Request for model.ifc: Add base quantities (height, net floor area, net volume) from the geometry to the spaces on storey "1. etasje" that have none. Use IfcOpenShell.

First a look at what the model holds.

```python
import ifcopenshell
import ifcopenshell.util.element
import ifcopenshell.util.unit

model = ifcopenshell.open("model.ifc")
print(model.schema)
for unit_type in ("LENGTHUNIT", "AREAUNIT", "VOLUMEUNIT"):
    print(unit_type, ifcopenshell.util.unit.calculate_unit_scale(model, unit_type))
storey = next(s for s in model.by_type("IfcBuildingStorey") if s.Name == "1. etasje")
spaces = [e for e in ifcopenshell.util.element.get_decomposition(storey) if e.is_a("IfcSpace")]
for e in sorted(spaces, key=lambda e: e.id()):
    print(e.id(), e.is_a(), e.Name, list(ifcopenshell.util.element.get_psets(e, qtos_only=True)), sep=" | ")
```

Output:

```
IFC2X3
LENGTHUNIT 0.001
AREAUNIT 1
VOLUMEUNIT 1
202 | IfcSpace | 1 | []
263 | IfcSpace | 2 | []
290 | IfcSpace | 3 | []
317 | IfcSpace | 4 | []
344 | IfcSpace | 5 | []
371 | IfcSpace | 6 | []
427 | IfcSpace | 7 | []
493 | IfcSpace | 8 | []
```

```python
import ifcopenshell
import ifcopenshell.api.pset
import ifcopenshell.geom
import ifcopenshell.util.element
import ifcopenshell.util.shape
import ifcopenshell.util.unit

model = ifcopenshell.open("model.ifc")
unit_scale = ifcopenshell.util.unit.calculate_unit_scale(model)
area_scale = ifcopenshell.util.unit.calculate_unit_scale(model, "AREAUNIT")
volume_scale = ifcopenshell.util.unit.calculate_unit_scale(model, "VOLUMEUNIT")
settings = ifcopenshell.geom.settings()

storey = next(s for s in model.by_type("IfcBuildingStorey") if s.Name == "1. etasje")
spaces = [e for e in ifcopenshell.util.element.get_decomposition(storey) if e.is_a("IfcSpace")]

for e in sorted(spaces, key=lambda e: e.id()):
    if ifcopenshell.util.element.get_psets(e, qtos_only=True, should_inherit=False):
        continue
    # Geometry comes back in metres, in the element's own axes.
    shape = ifcopenshell.geom.create_shape(settings, e)
    values = {
        "Height": ifcopenshell.util.shape.get_z(shape.geometry) / unit_scale,
        "NetFloorArea": ifcopenshell.util.shape.get_footprint_area(shape.geometry) / area_scale,
        "NetVolume": ifcopenshell.util.shape.get_volume(shape.geometry) / volume_scale,
    }
    qto = ifcopenshell.api.pset.add_qto(model, product=e, name="BaseQuantities")
    ifcopenshell.api.pset.edit_qto(model, qto=qto, properties=values)
    print(e.id(), {k: round(v, 3) for k, v in values.items()})

model.write("model_edited.ifc")
```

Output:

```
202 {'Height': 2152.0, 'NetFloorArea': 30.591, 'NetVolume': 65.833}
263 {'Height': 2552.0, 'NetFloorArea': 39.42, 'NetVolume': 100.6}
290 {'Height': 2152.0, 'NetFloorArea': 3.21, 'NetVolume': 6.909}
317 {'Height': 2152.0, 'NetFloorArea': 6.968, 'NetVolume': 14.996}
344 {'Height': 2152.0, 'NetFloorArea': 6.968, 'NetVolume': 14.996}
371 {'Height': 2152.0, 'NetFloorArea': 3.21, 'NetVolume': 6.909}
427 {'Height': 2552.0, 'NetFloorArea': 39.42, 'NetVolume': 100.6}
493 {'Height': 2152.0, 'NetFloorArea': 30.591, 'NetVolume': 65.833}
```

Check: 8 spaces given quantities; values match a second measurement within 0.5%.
